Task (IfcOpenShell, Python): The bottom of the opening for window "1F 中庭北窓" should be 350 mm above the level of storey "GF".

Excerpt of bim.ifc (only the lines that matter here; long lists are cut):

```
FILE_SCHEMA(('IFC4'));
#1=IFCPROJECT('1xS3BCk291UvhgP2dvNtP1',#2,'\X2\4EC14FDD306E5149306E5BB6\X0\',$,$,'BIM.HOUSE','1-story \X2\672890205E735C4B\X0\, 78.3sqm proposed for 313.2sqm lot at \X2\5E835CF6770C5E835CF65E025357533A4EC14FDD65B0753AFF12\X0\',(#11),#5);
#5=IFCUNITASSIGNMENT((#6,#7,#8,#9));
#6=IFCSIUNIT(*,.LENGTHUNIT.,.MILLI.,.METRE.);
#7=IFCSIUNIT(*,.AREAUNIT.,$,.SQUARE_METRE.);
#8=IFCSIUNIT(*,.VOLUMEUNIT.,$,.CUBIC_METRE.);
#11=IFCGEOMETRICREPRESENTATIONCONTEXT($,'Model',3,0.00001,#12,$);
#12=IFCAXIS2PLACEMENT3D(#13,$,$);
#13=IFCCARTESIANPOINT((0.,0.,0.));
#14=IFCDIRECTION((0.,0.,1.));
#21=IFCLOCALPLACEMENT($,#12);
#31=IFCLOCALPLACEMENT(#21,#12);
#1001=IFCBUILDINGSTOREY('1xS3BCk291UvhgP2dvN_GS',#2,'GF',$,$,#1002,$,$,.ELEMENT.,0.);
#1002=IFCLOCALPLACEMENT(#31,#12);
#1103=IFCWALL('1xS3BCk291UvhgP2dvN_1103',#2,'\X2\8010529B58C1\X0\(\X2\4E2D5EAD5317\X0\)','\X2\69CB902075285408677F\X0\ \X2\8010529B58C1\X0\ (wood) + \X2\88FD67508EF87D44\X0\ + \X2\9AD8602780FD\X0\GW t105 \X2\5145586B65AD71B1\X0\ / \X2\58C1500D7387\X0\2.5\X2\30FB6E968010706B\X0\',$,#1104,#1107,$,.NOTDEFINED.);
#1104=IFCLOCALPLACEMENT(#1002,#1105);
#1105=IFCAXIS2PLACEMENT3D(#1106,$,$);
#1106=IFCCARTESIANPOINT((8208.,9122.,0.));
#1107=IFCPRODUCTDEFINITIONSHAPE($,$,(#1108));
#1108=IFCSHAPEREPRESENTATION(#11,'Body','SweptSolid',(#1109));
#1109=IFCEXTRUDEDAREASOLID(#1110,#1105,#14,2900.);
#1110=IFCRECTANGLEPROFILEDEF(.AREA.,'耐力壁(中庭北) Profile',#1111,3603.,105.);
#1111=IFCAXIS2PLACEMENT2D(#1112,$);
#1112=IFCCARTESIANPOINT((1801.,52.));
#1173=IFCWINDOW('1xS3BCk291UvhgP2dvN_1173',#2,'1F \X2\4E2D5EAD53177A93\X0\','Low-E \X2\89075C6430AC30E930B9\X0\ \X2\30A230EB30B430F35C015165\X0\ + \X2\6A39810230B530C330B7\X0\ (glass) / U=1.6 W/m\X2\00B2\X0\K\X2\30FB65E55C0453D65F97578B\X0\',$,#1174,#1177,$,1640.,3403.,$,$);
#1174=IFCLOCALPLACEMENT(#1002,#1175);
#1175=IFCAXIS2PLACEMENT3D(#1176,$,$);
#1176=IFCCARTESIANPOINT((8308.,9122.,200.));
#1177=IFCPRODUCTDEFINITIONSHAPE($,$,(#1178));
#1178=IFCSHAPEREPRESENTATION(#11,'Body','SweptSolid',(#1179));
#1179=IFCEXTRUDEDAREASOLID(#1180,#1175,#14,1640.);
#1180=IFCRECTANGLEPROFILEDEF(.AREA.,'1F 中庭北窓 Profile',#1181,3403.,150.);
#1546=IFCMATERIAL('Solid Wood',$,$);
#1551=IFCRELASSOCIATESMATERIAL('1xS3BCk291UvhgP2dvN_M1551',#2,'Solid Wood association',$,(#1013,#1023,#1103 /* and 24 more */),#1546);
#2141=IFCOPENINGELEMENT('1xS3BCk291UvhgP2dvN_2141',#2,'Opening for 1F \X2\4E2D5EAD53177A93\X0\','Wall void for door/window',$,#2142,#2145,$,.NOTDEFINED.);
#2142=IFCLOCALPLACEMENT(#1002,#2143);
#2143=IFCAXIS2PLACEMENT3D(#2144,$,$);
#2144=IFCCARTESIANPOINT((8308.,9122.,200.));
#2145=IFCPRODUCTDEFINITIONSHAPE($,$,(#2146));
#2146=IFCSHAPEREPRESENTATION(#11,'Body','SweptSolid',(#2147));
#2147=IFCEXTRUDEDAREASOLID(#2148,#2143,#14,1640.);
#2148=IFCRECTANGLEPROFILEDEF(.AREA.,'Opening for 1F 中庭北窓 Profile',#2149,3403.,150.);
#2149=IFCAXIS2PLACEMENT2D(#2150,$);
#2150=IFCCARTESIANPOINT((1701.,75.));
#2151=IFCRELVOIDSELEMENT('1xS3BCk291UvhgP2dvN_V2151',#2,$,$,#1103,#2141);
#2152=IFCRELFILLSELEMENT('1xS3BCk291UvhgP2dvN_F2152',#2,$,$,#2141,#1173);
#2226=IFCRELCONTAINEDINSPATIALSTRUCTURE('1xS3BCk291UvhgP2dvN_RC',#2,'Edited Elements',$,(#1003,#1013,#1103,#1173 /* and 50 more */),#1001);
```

```python
import numpy as np
import ifcopenshell
import ifcopenshell.api.geometry
import ifcopenshell.geom
import ifcopenshell.util.element
import ifcopenshell.util.placement
import ifcopenshell.util.shape
import ifcopenshell.util.unit

model = ifcopenshell.open("bim.ifc")
unit_scale = ifcopenshell.util.unit.calculate_unit_scale(model)

window = model.by_id(1173)
opening = window.FillsVoids[0].RelatingOpeningElement
storey = ifcopenshell.util.element.get_container(window, ifc_class="IfcBuildingStorey")
level = ifcopenshell.util.placement.get_local_placement(storey.ObjectPlacement)[2, 3]

# The opening's origin need not be at the sill, so measure its lowest point.
shape = ifcopenshell.geom.create_shape(ifcopenshell.geom.settings(), opening)
bottom = ifcopenshell.util.shape.get_shape_bottom_elevation(shape, shape.geometry) / unit_scale
dz = level + 0.35 / unit_scale - bottom

shift = np.array([0.0, 0.0, dz])
# The window is not placed relative to its opening, so move both.
for product in (opening, window):
    matrix = ifcopenshell.util.placement.get_local_placement(product.ObjectPlacement)
    matrix[:3, 3] += shift
    ifcopenshell.api.geometry.edit_object_placement(model, product=product, matrix=matrix, is_si=False)

print(f"moved by {dz * unit_scale:+.3f} m")

model.write("bim_rev.ifc")
```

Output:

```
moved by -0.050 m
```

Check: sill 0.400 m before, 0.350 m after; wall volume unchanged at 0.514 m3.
